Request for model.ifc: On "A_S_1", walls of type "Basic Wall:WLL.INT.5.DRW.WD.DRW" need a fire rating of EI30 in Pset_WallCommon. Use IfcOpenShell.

First a look at what the model holds.

```python
import ifcopenshell
import ifcopenshell.util.element

model = ifcopenshell.open("model.ifc")
print(model.schema)
storey = next(s for s in model.by_type("IfcBuildingStorey") if s.Name == "A_S_1")
walls = [e for e in ifcopenshell.util.element.get_decomposition(storey) if e.is_a("IfcWall")]
seen = {}
for e in walls:
    element_type = ifcopenshell.util.element.get_type(e)
    key = (element_type.Name if element_type != e and element_type else None, ifcopenshell.util.element.get_pset(e, "Pset_WallCommon", "FireRating"))
    seen[key] = seen.get(key, 0) + 1
for (name, value), count in sorted(seen.items(), key=str):
    print(count, "x", name, "|", value)
```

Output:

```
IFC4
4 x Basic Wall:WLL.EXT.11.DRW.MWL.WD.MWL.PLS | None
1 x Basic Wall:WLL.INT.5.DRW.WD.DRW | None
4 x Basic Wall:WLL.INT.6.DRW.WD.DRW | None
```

```python
import ifcopenshell
import ifcopenshell.api.pset
import ifcopenshell.util.element

model = ifcopenshell.open("model.ifc")

storey = next(s for s in model.by_type("IfcBuildingStorey") if s.Name == "A_S_1")
walls = [e for e in ifcopenshell.util.element.get_decomposition(storey) if e.is_a("IfcWall")]

count = 0
for e in walls:
    element_type = ifcopenshell.util.element.get_type(e)
    if element_type in (None, e) or element_type.Name != "Basic Wall:WLL.INT.5.DRW.WD.DRW":
        continue
    # add_pset returns the element's existing set when there is one.
    pset = ifcopenshell.api.pset.add_pset(model, product=e, name="Pset_WallCommon")
    ifcopenshell.api.pset.edit_pset(model, pset=pset, properties={"FireRating": "EI30"})
    count += 1

print(count, "walls updated")

model.write("model-out.ifc")
```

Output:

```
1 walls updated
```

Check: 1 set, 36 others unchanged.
